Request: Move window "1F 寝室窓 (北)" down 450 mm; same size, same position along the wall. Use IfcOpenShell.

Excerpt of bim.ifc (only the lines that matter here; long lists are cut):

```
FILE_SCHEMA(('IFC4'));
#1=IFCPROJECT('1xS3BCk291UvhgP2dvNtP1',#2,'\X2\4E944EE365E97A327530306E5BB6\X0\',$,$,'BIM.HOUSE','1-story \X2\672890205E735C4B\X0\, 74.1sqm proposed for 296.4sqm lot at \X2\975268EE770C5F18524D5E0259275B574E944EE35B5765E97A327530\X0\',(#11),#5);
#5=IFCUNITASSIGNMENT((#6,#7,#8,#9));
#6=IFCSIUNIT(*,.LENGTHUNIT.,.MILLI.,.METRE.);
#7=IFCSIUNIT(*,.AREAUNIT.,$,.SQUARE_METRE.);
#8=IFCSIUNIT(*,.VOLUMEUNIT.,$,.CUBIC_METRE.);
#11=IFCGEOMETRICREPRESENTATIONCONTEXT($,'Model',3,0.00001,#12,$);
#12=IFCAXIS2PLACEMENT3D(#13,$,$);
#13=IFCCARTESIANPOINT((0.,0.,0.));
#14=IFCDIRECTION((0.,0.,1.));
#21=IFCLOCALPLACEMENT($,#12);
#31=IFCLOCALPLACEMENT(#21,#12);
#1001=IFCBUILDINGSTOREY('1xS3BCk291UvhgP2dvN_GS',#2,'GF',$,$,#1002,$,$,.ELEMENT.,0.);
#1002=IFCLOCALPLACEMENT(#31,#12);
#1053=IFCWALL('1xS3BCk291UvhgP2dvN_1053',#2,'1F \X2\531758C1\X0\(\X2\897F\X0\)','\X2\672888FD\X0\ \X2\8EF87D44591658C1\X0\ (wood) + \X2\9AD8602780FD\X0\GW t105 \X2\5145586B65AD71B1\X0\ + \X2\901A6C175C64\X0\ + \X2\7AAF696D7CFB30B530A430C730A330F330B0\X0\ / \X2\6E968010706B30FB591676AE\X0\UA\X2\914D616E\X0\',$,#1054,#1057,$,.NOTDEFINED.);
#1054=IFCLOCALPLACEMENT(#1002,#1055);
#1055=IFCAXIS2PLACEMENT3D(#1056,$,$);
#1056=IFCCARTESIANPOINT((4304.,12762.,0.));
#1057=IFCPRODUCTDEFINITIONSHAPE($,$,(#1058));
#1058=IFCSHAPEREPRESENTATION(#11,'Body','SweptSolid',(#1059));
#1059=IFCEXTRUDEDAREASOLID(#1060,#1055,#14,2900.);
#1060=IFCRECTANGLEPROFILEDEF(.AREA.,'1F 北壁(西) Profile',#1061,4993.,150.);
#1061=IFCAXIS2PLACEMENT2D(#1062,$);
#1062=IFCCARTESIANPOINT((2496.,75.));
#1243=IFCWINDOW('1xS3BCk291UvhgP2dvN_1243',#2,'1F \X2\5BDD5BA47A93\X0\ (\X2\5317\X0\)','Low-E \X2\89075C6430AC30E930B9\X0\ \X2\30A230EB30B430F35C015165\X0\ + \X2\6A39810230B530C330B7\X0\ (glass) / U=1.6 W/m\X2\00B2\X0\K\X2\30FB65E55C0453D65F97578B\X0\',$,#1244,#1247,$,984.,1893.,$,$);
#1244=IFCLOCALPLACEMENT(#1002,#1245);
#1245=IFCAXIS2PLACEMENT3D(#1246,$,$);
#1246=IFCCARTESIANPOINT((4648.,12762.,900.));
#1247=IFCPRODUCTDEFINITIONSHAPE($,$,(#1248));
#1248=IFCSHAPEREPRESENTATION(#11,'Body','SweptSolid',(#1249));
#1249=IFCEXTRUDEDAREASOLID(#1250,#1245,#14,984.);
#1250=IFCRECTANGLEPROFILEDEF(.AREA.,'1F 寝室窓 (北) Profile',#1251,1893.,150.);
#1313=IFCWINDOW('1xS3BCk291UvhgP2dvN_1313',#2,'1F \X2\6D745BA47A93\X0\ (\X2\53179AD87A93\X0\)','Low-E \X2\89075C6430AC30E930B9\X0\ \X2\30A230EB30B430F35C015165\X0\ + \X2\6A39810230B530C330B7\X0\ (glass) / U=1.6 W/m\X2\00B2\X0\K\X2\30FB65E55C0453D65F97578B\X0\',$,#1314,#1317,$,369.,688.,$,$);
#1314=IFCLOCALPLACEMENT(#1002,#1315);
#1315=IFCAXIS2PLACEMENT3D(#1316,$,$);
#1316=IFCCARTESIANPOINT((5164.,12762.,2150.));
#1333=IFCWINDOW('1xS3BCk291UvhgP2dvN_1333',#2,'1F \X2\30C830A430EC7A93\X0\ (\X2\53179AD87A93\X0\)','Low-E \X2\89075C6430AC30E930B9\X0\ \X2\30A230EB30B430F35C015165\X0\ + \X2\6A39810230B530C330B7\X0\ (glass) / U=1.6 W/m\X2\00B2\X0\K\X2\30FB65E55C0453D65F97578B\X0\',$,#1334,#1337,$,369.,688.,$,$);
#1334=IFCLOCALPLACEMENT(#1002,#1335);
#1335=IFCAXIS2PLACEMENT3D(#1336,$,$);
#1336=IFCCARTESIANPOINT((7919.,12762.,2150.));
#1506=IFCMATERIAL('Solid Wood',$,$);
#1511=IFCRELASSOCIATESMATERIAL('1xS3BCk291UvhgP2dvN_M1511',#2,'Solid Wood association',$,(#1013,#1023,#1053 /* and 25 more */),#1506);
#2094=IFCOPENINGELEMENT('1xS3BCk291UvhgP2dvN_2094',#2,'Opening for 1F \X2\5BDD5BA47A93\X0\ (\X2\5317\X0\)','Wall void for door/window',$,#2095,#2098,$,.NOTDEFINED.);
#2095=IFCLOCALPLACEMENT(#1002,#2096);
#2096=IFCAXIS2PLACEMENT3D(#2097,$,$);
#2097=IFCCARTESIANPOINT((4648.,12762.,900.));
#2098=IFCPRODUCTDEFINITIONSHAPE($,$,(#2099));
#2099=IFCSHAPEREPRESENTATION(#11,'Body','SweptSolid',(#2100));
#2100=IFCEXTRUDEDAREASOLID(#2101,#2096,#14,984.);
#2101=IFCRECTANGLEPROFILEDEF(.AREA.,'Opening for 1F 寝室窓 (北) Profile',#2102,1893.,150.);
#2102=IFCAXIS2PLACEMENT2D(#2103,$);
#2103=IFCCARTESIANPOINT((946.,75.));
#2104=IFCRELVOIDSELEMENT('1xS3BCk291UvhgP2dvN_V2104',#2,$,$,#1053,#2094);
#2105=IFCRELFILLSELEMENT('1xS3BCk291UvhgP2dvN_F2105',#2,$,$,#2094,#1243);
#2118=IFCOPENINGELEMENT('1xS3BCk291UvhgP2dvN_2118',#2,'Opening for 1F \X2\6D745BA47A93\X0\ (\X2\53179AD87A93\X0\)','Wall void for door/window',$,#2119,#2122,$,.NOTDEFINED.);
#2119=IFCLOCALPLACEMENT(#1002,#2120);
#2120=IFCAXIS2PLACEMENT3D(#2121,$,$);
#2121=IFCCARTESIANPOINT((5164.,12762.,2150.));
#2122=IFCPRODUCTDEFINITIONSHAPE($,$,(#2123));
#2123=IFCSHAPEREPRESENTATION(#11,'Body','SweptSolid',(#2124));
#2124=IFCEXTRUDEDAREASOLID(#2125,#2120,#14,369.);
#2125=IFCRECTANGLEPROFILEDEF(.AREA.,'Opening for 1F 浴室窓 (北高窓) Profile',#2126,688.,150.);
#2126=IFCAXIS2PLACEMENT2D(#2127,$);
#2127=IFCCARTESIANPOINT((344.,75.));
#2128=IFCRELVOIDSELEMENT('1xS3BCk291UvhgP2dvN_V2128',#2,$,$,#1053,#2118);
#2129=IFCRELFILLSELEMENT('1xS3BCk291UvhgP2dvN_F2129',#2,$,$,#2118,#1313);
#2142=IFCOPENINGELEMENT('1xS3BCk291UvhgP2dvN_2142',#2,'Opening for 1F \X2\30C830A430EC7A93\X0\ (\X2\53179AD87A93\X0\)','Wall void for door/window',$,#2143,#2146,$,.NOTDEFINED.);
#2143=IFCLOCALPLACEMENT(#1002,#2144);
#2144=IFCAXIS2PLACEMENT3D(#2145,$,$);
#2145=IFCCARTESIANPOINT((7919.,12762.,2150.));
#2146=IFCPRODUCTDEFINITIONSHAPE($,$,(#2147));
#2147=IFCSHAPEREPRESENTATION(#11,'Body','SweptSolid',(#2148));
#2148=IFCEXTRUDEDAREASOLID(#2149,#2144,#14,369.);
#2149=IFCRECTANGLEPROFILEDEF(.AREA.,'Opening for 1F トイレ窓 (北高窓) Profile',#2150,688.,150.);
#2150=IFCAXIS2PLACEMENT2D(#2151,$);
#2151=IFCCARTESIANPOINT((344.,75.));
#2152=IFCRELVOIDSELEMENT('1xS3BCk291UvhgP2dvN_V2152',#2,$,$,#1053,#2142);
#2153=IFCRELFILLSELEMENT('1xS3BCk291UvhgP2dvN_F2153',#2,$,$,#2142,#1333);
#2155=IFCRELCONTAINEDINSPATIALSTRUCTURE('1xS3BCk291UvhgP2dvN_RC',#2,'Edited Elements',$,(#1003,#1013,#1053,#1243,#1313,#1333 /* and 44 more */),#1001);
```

```python
import numpy as np
import ifcopenshell
import ifcopenshell.api.geometry
import ifcopenshell.util.placement
import ifcopenshell.util.unit

model = ifcopenshell.open("bim.ifc")
unit_scale = ifcopenshell.util.unit.calculate_unit_scale(model)

window = model.by_guid("1xS3BCk291UvhgP2dvN_1243")
opening = window.FillsVoids[0].RelatingOpeningElement
dz = -0.45 / unit_scale

shift = np.array([0.0, 0.0, dz])
# The window is not placed relative to its opening, so move both.
for product in (opening, window):
    matrix = ifcopenshell.util.placement.get_local_placement(product.ObjectPlacement)
    matrix[:3, 3] += shift
    ifcopenshell.api.geometry.edit_object_placement(model, product=product, matrix=matrix, is_si=False)

print(f"moved by {dz * unit_scale:+.3f} m")

model.write("bim_updated.ifc")
```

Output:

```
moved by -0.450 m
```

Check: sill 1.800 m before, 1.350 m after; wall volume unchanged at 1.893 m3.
